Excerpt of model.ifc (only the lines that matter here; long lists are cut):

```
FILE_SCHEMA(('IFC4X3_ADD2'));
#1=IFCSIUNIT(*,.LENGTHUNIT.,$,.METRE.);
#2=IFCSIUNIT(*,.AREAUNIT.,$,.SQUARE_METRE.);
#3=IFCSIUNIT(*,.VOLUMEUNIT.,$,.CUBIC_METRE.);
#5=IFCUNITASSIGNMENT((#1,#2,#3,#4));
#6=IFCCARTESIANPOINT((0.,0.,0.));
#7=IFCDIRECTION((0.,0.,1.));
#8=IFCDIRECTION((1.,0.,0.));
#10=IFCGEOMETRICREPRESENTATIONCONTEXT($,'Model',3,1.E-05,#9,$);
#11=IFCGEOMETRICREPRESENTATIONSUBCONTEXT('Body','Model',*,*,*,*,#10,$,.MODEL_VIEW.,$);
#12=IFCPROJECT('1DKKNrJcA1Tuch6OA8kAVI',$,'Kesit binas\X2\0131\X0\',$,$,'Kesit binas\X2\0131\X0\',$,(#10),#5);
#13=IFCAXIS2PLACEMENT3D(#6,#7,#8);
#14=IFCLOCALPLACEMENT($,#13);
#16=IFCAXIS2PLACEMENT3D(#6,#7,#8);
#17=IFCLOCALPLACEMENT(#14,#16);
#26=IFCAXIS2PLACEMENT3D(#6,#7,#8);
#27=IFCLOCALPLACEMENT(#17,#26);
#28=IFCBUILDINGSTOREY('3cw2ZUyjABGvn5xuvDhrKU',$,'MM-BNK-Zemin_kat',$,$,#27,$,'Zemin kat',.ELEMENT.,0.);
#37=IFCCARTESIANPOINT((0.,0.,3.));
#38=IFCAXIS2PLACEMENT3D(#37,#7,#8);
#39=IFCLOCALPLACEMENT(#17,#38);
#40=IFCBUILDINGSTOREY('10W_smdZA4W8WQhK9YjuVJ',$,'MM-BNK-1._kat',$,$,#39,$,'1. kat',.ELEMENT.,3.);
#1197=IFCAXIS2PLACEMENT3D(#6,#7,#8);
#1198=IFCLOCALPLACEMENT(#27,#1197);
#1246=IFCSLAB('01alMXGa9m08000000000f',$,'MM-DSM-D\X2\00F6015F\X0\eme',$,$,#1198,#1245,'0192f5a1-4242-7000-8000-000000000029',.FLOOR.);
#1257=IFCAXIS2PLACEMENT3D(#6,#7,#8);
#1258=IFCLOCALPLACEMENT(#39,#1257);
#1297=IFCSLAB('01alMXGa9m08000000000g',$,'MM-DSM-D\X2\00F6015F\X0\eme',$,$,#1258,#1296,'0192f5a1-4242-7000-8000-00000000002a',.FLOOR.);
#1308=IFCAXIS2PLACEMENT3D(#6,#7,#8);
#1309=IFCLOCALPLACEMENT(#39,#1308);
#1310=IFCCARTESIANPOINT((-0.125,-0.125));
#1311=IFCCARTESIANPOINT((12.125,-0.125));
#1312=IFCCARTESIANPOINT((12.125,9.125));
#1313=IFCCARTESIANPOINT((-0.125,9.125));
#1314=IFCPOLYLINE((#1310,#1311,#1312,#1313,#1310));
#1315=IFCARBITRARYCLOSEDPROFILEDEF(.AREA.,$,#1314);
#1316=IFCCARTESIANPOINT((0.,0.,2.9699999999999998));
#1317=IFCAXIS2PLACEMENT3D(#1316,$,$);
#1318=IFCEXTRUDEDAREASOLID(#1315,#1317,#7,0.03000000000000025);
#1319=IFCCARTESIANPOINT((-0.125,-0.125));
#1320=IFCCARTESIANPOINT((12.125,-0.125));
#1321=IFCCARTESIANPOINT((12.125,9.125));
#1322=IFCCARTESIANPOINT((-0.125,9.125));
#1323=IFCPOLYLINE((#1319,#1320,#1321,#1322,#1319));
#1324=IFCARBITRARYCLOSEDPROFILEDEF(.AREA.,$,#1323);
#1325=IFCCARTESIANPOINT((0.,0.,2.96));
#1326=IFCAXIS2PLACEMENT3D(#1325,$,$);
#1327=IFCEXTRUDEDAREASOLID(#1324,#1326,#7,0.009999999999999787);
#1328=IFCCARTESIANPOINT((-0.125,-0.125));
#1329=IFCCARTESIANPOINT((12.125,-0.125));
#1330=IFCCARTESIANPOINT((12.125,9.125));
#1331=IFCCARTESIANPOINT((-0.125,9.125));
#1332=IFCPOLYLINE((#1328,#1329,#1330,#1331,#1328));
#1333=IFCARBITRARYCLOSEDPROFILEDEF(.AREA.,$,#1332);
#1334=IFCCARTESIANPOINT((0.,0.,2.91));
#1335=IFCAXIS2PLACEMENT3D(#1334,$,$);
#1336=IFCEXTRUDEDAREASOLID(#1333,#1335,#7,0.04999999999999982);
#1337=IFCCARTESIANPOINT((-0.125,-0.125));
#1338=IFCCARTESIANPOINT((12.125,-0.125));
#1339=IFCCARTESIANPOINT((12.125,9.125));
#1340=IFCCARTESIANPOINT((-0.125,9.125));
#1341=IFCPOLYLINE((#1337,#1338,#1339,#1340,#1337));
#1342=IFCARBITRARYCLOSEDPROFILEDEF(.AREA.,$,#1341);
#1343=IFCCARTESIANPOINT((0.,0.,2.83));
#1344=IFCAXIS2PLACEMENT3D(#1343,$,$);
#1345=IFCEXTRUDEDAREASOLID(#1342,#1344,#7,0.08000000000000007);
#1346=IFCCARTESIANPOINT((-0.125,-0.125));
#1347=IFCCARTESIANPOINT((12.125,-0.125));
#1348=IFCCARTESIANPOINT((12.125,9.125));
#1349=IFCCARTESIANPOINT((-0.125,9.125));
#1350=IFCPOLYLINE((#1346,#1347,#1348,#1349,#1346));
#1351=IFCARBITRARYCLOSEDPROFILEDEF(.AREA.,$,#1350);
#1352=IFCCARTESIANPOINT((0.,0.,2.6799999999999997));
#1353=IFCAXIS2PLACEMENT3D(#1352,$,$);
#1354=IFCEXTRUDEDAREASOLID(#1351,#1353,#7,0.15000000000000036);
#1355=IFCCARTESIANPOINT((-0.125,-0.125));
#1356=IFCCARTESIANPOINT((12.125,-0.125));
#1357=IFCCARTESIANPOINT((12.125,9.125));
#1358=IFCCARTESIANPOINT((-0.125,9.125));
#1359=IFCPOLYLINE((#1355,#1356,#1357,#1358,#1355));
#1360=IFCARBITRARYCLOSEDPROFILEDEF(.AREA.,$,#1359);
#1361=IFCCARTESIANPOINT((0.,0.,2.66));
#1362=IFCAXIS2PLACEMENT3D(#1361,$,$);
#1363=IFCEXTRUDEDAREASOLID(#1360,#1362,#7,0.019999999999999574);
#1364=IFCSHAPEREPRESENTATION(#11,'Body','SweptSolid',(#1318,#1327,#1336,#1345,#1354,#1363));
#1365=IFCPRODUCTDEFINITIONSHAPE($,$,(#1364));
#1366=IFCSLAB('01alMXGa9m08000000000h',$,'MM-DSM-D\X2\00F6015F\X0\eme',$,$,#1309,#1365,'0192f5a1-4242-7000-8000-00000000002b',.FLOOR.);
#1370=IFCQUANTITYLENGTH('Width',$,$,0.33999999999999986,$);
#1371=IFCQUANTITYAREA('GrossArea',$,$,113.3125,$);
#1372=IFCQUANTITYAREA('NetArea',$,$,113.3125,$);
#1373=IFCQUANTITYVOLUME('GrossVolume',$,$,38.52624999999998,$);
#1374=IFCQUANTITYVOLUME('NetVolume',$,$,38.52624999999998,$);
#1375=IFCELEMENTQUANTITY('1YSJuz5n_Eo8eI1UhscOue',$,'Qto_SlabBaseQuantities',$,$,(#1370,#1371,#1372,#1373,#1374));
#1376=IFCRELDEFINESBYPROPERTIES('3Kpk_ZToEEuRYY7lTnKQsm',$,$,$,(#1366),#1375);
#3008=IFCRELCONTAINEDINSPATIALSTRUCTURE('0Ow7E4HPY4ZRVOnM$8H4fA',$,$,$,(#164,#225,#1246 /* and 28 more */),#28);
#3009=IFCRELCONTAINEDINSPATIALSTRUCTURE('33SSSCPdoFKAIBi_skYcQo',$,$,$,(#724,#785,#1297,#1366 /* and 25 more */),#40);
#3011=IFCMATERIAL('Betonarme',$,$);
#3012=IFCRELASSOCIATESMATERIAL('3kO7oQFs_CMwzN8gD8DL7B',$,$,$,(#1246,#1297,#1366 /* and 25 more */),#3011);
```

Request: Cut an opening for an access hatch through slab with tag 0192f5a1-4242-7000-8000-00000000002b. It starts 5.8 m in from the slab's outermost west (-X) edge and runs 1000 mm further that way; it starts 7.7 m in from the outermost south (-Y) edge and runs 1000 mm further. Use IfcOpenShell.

```python
import numpy as np
import ifcopenshell
import ifcopenshell.api.feature
import ifcopenshell.api.geometry
import ifcopenshell.api.pset
import ifcopenshell.api.root
import ifcopenshell.geom
import ifcopenshell.util.element
import ifcopenshell.util.placement
import ifcopenshell.util.representation
import ifcopenshell.util.shape
import ifcopenshell.util.unit

model = ifcopenshell.open("model.ifc")
unit_scale = ifcopenshell.util.unit.calculate_unit_scale(model)
area_scale = ifcopenshell.util.unit.calculate_unit_scale(model, "AREAUNIT")
volume_scale = ifcopenshell.util.unit.calculate_unit_scale(model, "VOLUMEUNIT")
settings = ifcopenshell.geom.settings()


def volume(element):
    """Net volume in cubic metres, openings subtracted."""
    shape = ifcopenshell.geom.create_shape(settings, element)
    return ifcopenshell.util.shape.get_volume(shape.geometry)


slab = model.by_guid("01alMXGa9m08000000000h")
before = volume(slab)

# Extent in the slab's own axes, in metres. The edges named are its -X and -Y sides.
slab_shape = ifcopenshell.geom.create_shape(settings, slab)
vertices = ifcopenshell.util.shape.get_vertices(slab_shape.geometry)
x_min, y_min, bottom = vertices.min(axis=0)
top = vertices[:, 2].max()

opening = ifcopenshell.api.root.create_entity(model, ifc_class="IfcOpeningElement", name="Access hatch opening", predefined_type="OPENING")
context = ifcopenshell.util.representation.get_context(model, "Model", "Body", "MODEL_VIEW")
width, depth = 1, 1
outline = [(0.0, 0.0), (width, 0.0), (width, depth), (0.0, depth), (0.0, 0.0)]
# Overshoot both faces by 50 mm so the cut is clean.
shape = ifcopenshell.api.geometry.add_slab_representation(
    model, context=context, depth=top - bottom + 0.1, polyline=outline
)
ifcopenshell.api.geometry.assign_representation(model, product=opening, representation=shape)

matrix = ifcopenshell.util.placement.get_local_placement(slab.ObjectPlacement)
matrix[:, 3] = matrix @ np.append(np.array([x_min + 5.8, y_min + 7.7, bottom - 0.05]) / unit_scale, 1.0)
ifcopenshell.api.geometry.edit_object_placement(model, product=opening, matrix=matrix, is_si=False)
ifcopenshell.api.feature.add_feature(model, feature=opening, element=slab)

after = volume(slab)

# Update the slab's stored quantities.
qto = model.by_id(ifcopenshell.util.element.get_pset(slab, "Qto_SlabBaseQuantities", should_inherit=False)["id"])
ifcopenshell.api.pset.edit_qto(model, qto=qto, properties={
    "NetArea": after / (top - bottom) / area_scale,
    "NetVolume": after / volume_scale,
})

print(f"slab volume {before:.3f} -> {after:.3f} m3")

model.write("model-out.ifc")
```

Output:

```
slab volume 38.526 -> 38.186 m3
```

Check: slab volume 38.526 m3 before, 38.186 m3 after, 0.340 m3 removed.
